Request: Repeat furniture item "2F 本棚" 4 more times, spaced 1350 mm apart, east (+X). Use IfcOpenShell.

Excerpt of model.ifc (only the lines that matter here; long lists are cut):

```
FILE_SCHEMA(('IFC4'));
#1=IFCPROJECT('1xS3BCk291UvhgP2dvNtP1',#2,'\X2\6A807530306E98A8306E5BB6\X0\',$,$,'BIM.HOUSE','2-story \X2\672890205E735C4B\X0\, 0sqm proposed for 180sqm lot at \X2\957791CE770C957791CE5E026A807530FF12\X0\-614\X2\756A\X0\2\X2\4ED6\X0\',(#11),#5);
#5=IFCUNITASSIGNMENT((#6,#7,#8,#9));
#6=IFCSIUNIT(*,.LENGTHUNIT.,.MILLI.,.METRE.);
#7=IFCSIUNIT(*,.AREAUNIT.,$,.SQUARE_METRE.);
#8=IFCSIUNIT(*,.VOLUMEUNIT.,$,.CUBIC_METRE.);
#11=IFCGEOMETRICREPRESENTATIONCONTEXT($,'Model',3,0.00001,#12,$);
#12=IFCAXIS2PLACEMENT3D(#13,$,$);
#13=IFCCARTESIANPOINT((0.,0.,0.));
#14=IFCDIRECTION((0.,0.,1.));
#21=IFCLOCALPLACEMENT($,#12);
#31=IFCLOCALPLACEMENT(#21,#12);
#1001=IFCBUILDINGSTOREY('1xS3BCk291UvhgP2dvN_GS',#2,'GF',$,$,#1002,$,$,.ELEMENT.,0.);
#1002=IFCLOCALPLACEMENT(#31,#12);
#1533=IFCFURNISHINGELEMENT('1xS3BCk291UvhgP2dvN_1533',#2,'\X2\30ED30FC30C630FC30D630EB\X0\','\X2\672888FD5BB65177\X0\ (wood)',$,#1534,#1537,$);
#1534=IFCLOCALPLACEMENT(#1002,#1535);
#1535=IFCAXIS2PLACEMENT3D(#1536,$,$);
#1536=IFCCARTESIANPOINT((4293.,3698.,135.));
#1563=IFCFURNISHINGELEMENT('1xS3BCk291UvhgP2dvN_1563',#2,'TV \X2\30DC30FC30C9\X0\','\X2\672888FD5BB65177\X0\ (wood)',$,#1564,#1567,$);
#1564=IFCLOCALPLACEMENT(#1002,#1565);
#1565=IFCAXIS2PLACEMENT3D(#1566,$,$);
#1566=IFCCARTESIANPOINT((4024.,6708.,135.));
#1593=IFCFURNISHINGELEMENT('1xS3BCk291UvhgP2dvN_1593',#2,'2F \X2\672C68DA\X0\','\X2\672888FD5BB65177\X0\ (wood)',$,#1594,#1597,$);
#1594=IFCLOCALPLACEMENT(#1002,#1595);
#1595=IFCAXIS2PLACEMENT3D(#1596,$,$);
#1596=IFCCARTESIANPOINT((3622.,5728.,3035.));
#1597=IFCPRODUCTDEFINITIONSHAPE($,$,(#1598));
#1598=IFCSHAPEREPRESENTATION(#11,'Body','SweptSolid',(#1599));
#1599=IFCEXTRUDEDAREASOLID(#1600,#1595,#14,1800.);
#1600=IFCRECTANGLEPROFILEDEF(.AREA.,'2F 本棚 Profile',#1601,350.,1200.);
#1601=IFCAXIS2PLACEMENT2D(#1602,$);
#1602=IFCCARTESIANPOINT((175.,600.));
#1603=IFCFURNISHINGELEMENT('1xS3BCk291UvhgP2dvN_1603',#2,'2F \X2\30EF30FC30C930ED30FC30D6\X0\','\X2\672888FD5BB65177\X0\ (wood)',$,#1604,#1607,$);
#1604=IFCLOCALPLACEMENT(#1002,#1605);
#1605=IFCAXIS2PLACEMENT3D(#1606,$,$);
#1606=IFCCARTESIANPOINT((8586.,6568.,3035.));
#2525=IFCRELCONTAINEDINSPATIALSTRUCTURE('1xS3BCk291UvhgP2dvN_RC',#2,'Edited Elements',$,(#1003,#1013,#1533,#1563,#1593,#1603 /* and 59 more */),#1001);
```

```python
import numpy as np
import ifcopenshell
import ifcopenshell.api.geometry
import ifcopenshell.api.root
import ifcopenshell.util.element
import ifcopenshell.util.placement

model = ifcopenshell.open("model.ifc")


def reuse_history(source, copy):
    """copy_class also copies each property set's owner history, people and application; keep the originals."""
    for rel in copy.IsDefinedBy:
        if rel.is_a("IfcRelDefinesByProperties") and (history := rel.RelatingPropertyDefinition.OwnerHistory):
            rel.RelatingPropertyDefinition.OwnerHistory = source.OwnerHistory
            ifcopenshell.util.element.remove_deep2(model, history)


source = model.by_guid("1xS3BCk291UvhgP2dvN_1593")
base = ifcopenshell.util.placement.get_local_placement(source.ObjectPlacement)
step = np.array([1.0, 0.0, 0.0]) * 1350.0

for i in range(1, 5):
    copy = ifcopenshell.api.root.copy_class(model, product=source)
    copy.Representation = ifcopenshell.util.element.copy_deep(
        model, source.Representation, exclude=["IfcGeometricRepresentationContext", "IfcRepresentationMap"]
    )
    reuse_history(source, copy)
    matrix = base.copy()
    matrix[:3, 3] += i * step
    print("added at", matrix[:3, 3].round(3) + 0.0)
    ifcopenshell.api.geometry.edit_object_placement(model, product=copy, matrix=matrix, is_si=False)

model.write("model-out.ifc")
```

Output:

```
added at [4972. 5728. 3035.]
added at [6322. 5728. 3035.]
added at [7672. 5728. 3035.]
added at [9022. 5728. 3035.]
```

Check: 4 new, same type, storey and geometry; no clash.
